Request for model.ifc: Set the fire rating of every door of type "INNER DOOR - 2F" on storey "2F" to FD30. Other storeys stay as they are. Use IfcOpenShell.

First a look at what the model holds.

```python
import ifcopenshell
import ifcopenshell.util.element

model = ifcopenshell.open("model.ifc")
print(model.schema)
storey = next(s for s in model.by_type("IfcBuildingStorey") if s.Name == "2F")
doors = [e for e in ifcopenshell.util.element.get_decomposition(storey) if e.is_a("IfcDoor")]
seen = {}
for e in doors:
    element_type = ifcopenshell.util.element.get_type(e)
    key = (element_type.Name if element_type != e and element_type else None, ifcopenshell.util.element.get_pset(e, "Pset_DoorCommon", "FireRating"))
    seen[key] = seen.get(key, 0) + 1
for (name, value), count in sorted(seen.items(), key=str):
    print(count, "x", name, "|", value)
```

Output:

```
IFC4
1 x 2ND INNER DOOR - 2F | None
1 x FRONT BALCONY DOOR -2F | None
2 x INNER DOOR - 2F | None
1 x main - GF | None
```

```python
import ifcopenshell
import ifcopenshell.api.pset
import ifcopenshell.util.element

model = ifcopenshell.open("model.ifc")

storey = next(s for s in model.by_type("IfcBuildingStorey") if s.Name == "2F")
doors = [e for e in ifcopenshell.util.element.get_decomposition(storey) if e.is_a("IfcDoor")]

count = 0
for e in doors:
    element_type = ifcopenshell.util.element.get_type(e)
    if element_type in (None, e) or element_type.Name != "INNER DOOR - 2F":
        continue
    # add_pset returns the element's existing set when there is one.
    pset = ifcopenshell.api.pset.add_pset(model, product=e, name="Pset_DoorCommon")
    ifcopenshell.api.pset.edit_pset(model, pset=pset, properties={"FireRating": "FD30"})
    count += 1

print(count, "doors updated")

model.write("model_v2.ifc")
```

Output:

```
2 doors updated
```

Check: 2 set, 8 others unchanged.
